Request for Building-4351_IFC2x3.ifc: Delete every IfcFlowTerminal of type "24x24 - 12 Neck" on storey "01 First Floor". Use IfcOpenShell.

First a look at what the model holds.

```python
import ifcopenshell
import ifcopenshell.util.element

model = ifcopenshell.open("Building-4351_IFC2x3.ifc")
print(model.schema)
storey = next(s for s in model.by_type("IfcBuildingStorey") if s.Name == "01 First Floor")
terminals = [e for e in ifcopenshell.util.element.get_decomposition(storey) if e.is_a("IfcFlowTerminal")]
seen = {}
for e in terminals:
    element_type = ifcopenshell.util.element.get_type(e)
    name = element_type.Name if element_type not in (None, e) else None
    seen[name] = seen.get(name, 0) + 1
for name, count in sorted(seen.items(), key=str):
    print(count, "x", name)
```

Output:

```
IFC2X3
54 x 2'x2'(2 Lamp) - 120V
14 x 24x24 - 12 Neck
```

```python
import ifcopenshell
import ifcopenshell.api.root
import ifcopenshell.util.element

model = ifcopenshell.open("Building-4351_IFC2x3.ifc")

storey = next(s for s in model.by_type("IfcBuildingStorey") if s.Name == "01 First Floor")
terminals = [e for e in ifcopenshell.util.element.get_decomposition(storey) if e.is_a("IfcFlowTerminal")]
targets = [e for e in terminals if (t := ifcopenshell.util.element.get_type(e)) not in (None, e) and t.Name == "24x24 - 12 Neck"]

for e in targets:
    ifcopenshell.api.root.remove_product(model, product=e)
print(len(targets), "removed")

model.write("Building-4351_IFC2x3_rev.ifc")
```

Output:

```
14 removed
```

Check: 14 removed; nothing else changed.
